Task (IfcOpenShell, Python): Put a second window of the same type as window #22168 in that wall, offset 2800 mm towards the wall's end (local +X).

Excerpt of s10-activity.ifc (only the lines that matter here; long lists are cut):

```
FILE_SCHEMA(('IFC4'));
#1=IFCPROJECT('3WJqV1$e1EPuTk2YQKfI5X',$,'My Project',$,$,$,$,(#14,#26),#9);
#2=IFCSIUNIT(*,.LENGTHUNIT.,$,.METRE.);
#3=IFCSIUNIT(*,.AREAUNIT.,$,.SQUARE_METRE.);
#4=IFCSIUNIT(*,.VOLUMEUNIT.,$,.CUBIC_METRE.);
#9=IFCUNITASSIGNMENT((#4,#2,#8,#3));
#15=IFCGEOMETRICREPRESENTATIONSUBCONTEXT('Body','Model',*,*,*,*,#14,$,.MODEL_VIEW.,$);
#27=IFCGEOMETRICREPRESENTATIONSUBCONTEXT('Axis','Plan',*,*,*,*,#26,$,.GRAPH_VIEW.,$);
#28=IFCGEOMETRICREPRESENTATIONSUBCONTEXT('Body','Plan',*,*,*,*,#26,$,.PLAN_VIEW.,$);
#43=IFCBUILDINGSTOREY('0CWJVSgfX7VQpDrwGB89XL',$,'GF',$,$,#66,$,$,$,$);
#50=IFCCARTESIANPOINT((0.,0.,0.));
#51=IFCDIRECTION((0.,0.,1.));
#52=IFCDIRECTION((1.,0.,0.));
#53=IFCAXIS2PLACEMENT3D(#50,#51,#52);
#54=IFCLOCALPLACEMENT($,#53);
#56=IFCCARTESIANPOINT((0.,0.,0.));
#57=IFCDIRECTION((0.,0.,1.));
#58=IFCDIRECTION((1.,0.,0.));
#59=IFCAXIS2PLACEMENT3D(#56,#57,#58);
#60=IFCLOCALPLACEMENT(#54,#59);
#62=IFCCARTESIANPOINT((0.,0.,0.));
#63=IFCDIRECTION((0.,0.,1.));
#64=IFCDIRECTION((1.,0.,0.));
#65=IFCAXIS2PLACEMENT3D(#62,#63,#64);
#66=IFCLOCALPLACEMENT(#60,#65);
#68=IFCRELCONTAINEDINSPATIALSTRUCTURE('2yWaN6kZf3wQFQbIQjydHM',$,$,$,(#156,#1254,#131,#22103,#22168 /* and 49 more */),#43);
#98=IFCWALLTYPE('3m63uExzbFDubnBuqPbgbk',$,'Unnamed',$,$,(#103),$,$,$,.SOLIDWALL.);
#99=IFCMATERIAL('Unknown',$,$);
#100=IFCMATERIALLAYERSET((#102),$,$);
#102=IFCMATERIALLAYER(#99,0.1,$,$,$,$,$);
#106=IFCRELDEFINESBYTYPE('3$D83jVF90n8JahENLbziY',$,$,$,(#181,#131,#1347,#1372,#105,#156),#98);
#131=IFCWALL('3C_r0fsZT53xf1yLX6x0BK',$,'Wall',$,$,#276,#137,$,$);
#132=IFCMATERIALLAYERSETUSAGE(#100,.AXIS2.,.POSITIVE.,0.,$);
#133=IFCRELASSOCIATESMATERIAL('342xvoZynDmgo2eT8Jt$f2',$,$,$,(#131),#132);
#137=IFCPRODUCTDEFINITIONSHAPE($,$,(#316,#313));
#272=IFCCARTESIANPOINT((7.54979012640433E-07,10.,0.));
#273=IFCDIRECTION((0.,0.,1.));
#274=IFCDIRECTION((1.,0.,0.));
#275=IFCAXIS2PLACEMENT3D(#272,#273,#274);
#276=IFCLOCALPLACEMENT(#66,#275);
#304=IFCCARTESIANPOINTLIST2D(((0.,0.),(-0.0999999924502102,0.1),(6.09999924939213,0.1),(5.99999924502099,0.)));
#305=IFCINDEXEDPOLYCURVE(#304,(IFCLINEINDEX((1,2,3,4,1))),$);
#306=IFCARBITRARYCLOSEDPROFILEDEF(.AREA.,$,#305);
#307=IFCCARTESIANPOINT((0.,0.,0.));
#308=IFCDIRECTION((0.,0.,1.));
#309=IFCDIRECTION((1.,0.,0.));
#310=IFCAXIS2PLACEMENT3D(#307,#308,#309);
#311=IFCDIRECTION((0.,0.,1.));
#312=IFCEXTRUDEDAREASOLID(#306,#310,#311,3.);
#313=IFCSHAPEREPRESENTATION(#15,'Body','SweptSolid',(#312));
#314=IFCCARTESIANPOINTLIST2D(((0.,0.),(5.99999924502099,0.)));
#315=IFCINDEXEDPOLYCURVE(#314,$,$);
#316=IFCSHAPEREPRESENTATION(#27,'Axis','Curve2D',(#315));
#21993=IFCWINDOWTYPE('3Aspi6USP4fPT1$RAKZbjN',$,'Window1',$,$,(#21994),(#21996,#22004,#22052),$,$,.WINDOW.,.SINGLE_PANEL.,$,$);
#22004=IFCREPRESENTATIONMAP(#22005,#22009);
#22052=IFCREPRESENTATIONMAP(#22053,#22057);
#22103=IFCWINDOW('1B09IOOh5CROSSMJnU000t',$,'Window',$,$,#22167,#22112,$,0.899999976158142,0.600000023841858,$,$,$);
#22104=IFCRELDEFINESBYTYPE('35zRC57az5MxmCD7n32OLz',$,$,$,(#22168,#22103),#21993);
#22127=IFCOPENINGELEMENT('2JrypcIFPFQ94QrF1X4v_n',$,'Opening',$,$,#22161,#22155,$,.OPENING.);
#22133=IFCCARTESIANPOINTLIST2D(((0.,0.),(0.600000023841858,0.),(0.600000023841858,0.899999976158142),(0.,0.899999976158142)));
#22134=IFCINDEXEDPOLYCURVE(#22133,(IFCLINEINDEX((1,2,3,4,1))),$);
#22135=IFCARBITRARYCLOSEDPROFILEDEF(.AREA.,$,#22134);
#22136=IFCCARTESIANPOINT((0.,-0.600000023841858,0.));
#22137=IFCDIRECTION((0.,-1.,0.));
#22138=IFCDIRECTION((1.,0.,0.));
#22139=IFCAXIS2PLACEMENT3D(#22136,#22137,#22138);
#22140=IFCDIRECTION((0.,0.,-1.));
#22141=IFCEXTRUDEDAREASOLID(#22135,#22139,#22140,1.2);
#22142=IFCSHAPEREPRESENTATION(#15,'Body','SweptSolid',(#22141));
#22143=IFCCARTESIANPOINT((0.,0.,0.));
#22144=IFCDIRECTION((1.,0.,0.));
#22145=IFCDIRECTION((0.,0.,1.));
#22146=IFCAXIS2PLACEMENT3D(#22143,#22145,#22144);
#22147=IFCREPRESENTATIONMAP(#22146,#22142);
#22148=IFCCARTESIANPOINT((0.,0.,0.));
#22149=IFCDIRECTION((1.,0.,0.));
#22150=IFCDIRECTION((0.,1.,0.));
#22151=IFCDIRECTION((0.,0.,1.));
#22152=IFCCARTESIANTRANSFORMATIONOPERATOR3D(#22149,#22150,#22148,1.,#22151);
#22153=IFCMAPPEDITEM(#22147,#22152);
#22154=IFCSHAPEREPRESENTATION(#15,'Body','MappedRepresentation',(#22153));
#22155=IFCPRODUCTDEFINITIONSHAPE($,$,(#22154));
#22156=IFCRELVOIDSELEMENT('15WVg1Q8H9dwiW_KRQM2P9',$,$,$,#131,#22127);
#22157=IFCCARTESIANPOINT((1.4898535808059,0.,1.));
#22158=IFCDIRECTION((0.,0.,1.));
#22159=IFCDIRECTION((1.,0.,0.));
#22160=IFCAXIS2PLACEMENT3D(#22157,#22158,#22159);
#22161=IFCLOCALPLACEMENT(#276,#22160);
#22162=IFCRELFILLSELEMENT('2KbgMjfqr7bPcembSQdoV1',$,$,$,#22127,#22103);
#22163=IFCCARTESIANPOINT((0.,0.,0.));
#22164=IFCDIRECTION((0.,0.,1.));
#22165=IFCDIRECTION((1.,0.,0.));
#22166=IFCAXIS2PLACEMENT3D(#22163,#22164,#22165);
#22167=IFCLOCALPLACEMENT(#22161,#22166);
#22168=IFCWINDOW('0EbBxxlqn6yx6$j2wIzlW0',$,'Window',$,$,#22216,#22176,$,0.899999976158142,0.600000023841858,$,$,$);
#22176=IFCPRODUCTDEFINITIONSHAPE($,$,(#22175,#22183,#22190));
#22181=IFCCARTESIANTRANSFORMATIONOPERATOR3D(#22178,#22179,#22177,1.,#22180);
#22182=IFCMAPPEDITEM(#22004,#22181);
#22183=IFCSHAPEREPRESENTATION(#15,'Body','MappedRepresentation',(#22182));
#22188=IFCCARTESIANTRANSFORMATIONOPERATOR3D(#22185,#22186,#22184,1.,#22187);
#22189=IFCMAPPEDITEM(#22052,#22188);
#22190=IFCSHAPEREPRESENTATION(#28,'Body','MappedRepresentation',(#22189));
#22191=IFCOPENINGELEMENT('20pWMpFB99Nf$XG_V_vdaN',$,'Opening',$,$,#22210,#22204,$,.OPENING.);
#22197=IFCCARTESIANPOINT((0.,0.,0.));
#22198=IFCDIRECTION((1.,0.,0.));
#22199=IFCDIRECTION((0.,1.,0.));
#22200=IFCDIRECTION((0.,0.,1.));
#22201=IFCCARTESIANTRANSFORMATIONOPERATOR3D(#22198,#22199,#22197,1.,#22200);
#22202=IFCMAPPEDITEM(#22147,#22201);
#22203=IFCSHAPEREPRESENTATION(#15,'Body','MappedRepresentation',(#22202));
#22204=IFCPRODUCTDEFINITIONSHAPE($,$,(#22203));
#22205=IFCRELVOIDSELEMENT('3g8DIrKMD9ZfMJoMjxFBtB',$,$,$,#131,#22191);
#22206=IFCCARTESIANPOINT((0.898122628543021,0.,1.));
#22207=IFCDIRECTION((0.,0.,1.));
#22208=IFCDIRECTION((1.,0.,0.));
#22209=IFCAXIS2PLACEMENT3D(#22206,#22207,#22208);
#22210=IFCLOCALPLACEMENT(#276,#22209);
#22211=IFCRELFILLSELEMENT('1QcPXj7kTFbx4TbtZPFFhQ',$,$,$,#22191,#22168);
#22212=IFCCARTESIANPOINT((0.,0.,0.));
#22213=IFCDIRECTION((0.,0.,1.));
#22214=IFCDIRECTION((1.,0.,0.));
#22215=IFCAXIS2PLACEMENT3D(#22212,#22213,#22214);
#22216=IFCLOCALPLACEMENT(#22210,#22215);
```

```python
import ifcopenshell
import ifcopenshell.api.feature
import ifcopenshell.api.geometry
import ifcopenshell.api.root
import ifcopenshell.geom
import ifcopenshell.util.element
import ifcopenshell.util.placement
import ifcopenshell.util.shape
import ifcopenshell.util.unit

model = ifcopenshell.open("s10-activity.ifc")
unit_scale = ifcopenshell.util.unit.calculate_unit_scale(model)
settings = ifcopenshell.geom.settings()


def volume(element):
    """Net volume in cubic metres, openings subtracted."""
    shape = ifcopenshell.geom.create_shape(settings, element)
    return ifcopenshell.util.shape.get_volume(shape.geometry)


window = model.by_guid("0EbBxxlqn6yx6$j2wIzlW0")
opening = window.FillsVoids[0].RelatingOpeningElement
wall = opening.VoidsElements[0].RelatingBuildingElement
before = volume(wall)
shift = ifcopenshell.util.placement.get_local_placement(wall.ObjectPlacement)[:3, 0] * 2.8 / unit_scale

# copy_class copies the void relationship, type, container and properties, but no geometry.
new_opening = ifcopenshell.api.root.copy_class(model, product=opening)
new_opening.Representation = ifcopenshell.util.element.copy_deep(
    model, opening.Representation, exclude=["IfcGeometricRepresentationContext", "IfcRepresentationMap"]
)
new_window = ifcopenshell.api.root.copy_class(model, product=window)
new_window.Representation = ifcopenshell.util.element.copy_deep(
    model, window.Representation, exclude=["IfcGeometricRepresentationContext", "IfcRepresentationMap"]
)
ifcopenshell.api.feature.add_filling(model, opening=new_opening, element=new_window)

for old, new in ((opening, new_opening), (window, new_window)):
    matrix = ifcopenshell.util.placement.get_local_placement(old.ObjectPlacement)
    matrix[:3, 3] += shift
    ifcopenshell.api.geometry.edit_object_placement(model, product=new, matrix=matrix, is_si=False)

after = volume(wall)

print(f"wall volume {before:.3f} -> {after:.3f} m3")

model.write("s10-activity_v2.ifc")
```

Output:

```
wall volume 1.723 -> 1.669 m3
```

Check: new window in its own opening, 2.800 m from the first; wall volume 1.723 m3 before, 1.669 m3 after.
